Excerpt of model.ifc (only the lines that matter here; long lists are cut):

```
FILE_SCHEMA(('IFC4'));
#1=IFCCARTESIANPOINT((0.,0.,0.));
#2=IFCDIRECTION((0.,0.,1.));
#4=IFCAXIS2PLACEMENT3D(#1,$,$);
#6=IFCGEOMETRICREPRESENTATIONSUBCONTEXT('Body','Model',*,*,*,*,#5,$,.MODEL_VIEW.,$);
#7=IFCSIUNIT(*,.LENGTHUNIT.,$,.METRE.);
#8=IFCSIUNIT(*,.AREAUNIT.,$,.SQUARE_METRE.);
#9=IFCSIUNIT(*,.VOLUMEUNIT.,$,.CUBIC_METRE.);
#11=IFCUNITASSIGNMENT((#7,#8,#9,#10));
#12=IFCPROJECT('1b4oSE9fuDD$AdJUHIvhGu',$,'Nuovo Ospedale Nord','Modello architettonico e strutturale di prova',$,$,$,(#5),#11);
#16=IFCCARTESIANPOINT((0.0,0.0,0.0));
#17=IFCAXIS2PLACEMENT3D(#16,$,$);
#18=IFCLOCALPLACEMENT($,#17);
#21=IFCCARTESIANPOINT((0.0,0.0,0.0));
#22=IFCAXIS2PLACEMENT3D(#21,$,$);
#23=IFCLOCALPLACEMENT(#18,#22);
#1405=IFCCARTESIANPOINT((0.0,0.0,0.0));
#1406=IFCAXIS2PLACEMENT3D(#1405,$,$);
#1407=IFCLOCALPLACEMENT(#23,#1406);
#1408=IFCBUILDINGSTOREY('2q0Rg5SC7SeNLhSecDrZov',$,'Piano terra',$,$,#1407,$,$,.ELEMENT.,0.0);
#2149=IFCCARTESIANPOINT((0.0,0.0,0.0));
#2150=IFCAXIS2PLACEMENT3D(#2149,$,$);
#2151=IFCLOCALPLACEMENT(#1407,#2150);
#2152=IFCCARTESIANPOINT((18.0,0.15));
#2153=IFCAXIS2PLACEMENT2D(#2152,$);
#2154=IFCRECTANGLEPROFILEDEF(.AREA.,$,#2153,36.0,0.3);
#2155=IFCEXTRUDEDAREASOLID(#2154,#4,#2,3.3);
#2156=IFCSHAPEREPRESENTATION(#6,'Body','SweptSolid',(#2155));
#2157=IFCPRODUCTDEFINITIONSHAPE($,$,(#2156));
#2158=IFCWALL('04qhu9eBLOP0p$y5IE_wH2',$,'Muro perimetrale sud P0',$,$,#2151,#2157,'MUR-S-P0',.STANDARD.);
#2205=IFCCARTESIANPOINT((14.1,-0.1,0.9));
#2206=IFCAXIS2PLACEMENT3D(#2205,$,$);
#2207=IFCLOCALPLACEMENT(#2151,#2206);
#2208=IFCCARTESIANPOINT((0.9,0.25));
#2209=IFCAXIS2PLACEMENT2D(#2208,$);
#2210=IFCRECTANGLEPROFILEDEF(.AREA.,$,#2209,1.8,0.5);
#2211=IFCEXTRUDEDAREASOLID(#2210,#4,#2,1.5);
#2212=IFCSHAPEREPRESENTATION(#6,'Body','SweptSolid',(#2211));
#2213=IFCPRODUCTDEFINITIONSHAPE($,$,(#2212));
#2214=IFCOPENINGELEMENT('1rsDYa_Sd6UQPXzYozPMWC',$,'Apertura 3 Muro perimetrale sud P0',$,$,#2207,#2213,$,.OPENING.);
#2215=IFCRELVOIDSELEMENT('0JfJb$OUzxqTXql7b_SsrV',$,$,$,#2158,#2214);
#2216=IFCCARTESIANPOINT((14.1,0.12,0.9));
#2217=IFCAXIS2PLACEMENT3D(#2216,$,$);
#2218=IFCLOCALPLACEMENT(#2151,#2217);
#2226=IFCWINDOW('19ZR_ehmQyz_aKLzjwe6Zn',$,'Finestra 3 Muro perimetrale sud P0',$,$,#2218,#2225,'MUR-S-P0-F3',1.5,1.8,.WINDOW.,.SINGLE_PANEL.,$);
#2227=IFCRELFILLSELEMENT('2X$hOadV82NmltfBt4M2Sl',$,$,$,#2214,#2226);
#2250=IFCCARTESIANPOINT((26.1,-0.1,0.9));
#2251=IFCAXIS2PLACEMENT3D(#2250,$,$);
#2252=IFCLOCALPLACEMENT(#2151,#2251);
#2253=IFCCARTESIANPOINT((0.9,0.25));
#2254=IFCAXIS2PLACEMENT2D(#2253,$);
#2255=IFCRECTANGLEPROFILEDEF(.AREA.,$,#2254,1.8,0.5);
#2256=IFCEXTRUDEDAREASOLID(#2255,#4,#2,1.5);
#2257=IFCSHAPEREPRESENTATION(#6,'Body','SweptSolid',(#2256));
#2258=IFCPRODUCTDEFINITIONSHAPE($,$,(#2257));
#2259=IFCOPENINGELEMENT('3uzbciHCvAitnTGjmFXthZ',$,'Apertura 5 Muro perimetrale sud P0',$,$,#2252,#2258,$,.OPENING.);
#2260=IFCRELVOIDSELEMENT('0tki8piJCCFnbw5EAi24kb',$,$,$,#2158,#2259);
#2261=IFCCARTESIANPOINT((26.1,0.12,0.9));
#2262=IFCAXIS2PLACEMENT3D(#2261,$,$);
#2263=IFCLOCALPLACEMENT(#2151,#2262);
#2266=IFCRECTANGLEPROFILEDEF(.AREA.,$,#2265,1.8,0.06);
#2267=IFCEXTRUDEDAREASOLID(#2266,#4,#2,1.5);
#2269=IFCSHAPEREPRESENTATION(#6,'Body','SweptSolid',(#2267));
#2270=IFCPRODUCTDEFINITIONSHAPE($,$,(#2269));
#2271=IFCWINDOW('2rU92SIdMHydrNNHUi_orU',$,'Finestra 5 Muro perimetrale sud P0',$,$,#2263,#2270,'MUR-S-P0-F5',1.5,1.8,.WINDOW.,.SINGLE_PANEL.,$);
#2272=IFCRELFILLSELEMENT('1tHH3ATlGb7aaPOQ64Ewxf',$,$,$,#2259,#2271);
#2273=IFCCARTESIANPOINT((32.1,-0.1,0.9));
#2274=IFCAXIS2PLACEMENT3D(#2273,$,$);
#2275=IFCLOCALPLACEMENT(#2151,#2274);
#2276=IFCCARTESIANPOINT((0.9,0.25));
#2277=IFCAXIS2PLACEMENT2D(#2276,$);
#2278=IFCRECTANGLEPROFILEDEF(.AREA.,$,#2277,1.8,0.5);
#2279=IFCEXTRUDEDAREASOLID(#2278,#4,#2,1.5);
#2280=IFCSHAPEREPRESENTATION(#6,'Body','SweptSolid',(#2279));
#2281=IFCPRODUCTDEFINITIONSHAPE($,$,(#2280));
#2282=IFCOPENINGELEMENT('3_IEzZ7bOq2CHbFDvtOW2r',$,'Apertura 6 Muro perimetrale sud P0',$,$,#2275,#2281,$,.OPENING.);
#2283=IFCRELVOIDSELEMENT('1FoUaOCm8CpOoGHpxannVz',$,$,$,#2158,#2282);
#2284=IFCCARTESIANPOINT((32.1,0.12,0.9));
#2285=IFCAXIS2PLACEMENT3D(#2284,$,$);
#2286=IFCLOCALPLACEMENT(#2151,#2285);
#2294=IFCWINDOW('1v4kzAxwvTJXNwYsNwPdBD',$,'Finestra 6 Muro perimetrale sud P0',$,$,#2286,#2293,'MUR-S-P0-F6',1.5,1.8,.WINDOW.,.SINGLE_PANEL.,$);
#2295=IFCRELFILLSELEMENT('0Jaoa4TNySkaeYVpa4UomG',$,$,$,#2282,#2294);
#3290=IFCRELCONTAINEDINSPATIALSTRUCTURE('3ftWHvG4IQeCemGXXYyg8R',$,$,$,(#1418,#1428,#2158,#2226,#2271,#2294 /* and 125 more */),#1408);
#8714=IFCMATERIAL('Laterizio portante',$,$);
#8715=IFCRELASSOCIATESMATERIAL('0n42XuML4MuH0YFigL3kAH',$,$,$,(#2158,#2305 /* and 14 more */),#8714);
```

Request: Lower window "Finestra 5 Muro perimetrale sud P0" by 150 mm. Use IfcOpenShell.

```python
import numpy as np
import ifcopenshell
import ifcopenshell.api.geometry
import ifcopenshell.util.placement
import ifcopenshell.util.unit

model = ifcopenshell.open("model.ifc")
unit_scale = ifcopenshell.util.unit.calculate_unit_scale(model)

window = model.by_guid("2rU92SIdMHydrNNHUi_orU")
opening = window.FillsVoids[0].RelatingOpeningElement
dz = -0.15 / unit_scale

shift = np.array([0.0, 0.0, dz])
# The window is not placed relative to its opening, so move both.
for product in (opening, window):
    matrix = ifcopenshell.util.placement.get_local_placement(product.ObjectPlacement)
    matrix[:3, 3] += shift
    ifcopenshell.api.geometry.edit_object_placement(model, product=product, matrix=matrix, is_si=False)

print(f"moved by {dz * unit_scale:+.3f} m")

model.write("model_updated.ifc")
```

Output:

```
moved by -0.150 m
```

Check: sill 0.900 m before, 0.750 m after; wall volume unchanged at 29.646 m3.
